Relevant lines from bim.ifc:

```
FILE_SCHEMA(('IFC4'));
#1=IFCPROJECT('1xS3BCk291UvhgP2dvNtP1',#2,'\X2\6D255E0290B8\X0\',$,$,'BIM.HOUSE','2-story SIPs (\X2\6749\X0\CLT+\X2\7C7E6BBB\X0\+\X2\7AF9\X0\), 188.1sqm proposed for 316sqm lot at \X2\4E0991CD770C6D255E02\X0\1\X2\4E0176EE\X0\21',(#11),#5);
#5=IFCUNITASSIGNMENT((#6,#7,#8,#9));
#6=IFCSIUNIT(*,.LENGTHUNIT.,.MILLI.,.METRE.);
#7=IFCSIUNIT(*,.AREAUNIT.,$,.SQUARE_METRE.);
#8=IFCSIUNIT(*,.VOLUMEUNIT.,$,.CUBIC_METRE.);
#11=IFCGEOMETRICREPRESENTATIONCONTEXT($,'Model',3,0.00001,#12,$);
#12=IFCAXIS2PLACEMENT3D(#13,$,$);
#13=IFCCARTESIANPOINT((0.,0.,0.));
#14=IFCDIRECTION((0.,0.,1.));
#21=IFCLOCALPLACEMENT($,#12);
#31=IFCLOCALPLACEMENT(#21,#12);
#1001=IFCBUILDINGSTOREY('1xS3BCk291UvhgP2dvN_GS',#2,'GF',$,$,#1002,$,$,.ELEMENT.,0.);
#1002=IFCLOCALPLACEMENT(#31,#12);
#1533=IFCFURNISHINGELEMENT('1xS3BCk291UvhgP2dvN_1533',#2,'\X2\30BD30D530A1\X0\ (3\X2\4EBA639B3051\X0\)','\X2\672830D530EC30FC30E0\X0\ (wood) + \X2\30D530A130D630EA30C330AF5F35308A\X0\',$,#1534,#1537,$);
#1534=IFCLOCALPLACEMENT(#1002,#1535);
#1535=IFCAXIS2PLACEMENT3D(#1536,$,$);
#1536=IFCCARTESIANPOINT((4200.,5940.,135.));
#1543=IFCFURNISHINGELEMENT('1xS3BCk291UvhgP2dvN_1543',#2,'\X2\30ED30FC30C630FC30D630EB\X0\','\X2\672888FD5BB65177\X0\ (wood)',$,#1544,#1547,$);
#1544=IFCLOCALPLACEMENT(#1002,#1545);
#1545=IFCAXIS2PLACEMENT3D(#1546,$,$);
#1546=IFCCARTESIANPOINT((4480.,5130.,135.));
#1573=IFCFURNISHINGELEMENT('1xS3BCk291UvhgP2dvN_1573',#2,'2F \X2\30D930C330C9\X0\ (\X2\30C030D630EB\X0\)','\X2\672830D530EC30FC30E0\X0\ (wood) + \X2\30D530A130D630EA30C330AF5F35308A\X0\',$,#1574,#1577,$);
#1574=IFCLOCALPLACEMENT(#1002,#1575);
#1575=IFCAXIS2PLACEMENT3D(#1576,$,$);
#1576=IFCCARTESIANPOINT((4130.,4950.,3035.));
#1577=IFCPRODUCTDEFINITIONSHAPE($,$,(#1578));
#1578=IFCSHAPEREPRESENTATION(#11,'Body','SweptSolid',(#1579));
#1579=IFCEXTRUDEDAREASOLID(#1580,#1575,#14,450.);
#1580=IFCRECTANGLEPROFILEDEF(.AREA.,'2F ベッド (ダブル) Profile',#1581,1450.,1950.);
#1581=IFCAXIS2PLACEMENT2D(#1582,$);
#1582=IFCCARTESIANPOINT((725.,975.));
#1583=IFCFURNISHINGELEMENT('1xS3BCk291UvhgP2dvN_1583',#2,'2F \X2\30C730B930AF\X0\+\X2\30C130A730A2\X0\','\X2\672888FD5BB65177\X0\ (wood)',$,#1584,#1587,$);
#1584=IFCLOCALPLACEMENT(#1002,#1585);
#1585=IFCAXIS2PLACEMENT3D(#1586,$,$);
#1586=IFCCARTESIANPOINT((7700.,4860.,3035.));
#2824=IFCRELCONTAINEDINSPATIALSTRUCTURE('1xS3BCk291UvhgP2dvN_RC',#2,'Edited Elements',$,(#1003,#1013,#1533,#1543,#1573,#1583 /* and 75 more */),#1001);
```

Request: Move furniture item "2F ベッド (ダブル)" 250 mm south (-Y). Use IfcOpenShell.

```python
import ifcopenshell
import ifcopenshell.api.geometry
import ifcopenshell.util.placement
import ifcopenshell.util.unit

model = ifcopenshell.open("bim.ifc")
unit_scale = ifcopenshell.util.unit.calculate_unit_scale(model)

item = model.by_guid("1xS3BCk291UvhgP2dvN_1573")
matrix = ifcopenshell.util.placement.get_local_placement(item.ObjectPlacement)
matrix[1, 3] -= 0.25 / unit_scale
ifcopenshell.api.geometry.edit_object_placement(model, product=item, matrix=matrix, is_si=False)

print(ifcopenshell.util.placement.get_local_placement(item.ObjectPlacement).round(3) + 0.0)

model.write("bim_v2.ifc")
```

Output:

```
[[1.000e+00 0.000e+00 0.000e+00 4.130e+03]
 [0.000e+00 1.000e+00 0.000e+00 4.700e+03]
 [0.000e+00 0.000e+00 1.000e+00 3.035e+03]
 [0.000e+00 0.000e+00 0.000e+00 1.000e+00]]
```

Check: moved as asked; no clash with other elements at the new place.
